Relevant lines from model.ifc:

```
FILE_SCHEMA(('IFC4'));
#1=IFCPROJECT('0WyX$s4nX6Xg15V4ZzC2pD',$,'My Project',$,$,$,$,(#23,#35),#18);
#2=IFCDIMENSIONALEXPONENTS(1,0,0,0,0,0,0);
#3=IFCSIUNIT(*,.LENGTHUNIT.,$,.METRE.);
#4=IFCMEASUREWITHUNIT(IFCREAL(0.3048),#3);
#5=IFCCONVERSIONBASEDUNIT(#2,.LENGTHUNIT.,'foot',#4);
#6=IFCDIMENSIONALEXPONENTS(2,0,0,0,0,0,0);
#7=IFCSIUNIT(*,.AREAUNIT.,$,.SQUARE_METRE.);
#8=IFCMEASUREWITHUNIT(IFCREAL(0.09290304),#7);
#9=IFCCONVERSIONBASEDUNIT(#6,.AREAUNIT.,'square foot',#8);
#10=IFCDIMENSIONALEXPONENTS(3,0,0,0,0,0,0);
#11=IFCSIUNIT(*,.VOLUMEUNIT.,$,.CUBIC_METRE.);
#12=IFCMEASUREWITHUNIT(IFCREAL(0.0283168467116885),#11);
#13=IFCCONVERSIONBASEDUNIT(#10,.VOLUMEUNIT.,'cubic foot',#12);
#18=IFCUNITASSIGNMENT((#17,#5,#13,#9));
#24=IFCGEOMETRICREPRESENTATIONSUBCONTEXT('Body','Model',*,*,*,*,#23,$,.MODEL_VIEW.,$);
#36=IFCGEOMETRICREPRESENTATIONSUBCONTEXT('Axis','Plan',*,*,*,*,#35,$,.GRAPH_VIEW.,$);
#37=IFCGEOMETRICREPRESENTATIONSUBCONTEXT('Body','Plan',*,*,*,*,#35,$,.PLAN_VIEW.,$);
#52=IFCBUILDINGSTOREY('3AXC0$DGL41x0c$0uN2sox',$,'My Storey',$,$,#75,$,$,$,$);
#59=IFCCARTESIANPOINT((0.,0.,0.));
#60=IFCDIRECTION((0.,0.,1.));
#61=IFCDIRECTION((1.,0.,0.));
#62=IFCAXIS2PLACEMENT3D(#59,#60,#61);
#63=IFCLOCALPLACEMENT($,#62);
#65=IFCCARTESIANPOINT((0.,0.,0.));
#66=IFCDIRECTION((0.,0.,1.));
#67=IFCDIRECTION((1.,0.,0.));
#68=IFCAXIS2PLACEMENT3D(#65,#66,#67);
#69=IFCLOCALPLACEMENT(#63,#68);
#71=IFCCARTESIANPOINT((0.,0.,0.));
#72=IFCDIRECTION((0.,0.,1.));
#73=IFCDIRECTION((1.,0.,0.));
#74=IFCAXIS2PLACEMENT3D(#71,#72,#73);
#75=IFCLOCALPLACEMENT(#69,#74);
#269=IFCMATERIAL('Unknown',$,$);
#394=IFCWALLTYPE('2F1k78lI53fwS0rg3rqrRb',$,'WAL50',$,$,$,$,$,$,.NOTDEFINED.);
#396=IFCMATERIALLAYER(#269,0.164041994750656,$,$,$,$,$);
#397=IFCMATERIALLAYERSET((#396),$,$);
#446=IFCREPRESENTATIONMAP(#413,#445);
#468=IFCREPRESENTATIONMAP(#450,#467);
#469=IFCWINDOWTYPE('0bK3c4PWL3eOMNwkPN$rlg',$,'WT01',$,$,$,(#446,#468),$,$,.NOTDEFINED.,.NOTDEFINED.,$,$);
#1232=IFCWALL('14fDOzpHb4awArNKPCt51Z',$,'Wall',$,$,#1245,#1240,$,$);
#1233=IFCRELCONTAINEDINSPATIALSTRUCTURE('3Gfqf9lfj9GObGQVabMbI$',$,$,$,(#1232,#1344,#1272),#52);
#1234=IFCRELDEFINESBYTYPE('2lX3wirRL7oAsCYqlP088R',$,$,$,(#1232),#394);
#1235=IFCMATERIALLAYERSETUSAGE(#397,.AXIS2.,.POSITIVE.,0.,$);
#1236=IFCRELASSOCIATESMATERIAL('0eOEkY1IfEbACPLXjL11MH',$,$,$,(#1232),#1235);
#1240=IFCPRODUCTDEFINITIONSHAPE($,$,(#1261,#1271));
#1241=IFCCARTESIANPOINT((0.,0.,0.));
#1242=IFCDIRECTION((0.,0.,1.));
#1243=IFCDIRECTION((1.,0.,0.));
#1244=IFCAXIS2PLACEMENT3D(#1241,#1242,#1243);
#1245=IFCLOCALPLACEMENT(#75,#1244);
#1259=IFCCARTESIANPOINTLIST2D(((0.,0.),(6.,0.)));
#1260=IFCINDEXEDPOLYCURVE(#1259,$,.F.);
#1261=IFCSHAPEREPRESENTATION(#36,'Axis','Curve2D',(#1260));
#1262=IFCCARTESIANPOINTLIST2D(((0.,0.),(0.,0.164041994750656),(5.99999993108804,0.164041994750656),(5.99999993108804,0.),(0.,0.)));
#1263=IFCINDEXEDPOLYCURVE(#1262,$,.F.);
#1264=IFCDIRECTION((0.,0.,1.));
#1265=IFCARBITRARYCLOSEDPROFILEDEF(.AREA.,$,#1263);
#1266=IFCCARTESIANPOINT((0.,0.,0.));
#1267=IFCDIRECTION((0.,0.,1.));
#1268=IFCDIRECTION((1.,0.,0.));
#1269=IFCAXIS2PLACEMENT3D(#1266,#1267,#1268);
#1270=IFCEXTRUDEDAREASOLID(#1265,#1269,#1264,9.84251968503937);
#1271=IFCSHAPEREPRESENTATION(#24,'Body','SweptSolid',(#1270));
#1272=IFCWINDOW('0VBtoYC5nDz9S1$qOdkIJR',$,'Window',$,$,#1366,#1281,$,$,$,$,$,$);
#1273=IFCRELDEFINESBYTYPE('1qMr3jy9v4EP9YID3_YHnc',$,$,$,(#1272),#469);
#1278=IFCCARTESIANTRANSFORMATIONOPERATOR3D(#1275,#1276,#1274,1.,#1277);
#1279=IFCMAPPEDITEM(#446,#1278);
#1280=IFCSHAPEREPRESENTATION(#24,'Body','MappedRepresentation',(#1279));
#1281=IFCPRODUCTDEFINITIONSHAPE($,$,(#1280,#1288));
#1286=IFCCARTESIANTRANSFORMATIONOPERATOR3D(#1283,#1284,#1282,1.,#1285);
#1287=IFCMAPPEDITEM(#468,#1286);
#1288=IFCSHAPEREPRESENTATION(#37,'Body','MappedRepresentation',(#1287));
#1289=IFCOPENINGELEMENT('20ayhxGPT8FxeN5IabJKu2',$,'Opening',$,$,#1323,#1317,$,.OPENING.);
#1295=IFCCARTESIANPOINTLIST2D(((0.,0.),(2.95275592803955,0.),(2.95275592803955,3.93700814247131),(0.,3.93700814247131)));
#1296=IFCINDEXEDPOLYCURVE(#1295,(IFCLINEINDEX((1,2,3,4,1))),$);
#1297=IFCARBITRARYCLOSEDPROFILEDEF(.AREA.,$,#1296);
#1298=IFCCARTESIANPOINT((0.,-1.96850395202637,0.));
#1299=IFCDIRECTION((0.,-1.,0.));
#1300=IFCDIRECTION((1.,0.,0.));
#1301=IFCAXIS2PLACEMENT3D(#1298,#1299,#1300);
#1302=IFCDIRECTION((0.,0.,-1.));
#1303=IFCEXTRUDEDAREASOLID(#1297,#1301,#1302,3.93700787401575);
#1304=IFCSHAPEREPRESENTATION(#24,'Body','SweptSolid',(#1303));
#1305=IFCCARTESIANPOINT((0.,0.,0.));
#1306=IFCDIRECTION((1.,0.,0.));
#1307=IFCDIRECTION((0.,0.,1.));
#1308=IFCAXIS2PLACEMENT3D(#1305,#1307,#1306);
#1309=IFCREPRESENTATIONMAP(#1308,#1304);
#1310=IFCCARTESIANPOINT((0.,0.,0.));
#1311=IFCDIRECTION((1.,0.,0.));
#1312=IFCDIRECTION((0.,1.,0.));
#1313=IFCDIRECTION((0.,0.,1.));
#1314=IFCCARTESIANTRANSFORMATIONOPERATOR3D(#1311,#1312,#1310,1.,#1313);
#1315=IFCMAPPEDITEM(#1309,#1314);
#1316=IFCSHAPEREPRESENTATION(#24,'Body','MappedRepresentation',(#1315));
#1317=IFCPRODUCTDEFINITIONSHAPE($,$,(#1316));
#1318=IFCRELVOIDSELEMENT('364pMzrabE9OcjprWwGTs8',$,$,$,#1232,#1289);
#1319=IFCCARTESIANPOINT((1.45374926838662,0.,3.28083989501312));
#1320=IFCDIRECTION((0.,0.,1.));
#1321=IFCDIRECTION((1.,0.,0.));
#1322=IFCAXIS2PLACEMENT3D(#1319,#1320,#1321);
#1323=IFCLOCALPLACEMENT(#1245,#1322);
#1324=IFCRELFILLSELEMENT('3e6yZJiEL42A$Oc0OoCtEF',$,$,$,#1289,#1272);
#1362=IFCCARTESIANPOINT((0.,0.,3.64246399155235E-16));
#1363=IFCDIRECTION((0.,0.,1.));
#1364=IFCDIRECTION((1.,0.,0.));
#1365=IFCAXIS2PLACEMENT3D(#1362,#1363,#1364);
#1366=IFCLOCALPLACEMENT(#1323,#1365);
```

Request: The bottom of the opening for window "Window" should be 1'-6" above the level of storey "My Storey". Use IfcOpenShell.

```python
import numpy as np
import ifcopenshell
import ifcopenshell.api.geometry
import ifcopenshell.geom
import ifcopenshell.util.element
import ifcopenshell.util.placement
import ifcopenshell.util.shape
import ifcopenshell.util.unit

model = ifcopenshell.open("model.ifc")
unit_scale = ifcopenshell.util.unit.calculate_unit_scale(model)

window = model.by_guid("0VBtoYC5nDz9S1$qOdkIJR")
opening = window.FillsVoids[0].RelatingOpeningElement
storey = ifcopenshell.util.element.get_container(window, ifc_class="IfcBuildingStorey")
level = ifcopenshell.util.placement.get_local_placement(storey.ObjectPlacement)[2, 3]

# The opening's origin need not be at the sill, so measure its lowest point.
shape = ifcopenshell.geom.create_shape(ifcopenshell.geom.settings(), opening)
bottom = ifcopenshell.util.shape.get_shape_bottom_elevation(shape, shape.geometry) / unit_scale
dz = level + 18 * 0.0254 / unit_scale - bottom

shift = np.array([0.0, 0.0, dz])
# The window is placed relative to its opening, so it follows when the opening moves.
matrix = ifcopenshell.util.placement.get_local_placement(opening.ObjectPlacement)
matrix[:3, 3] += shift
ifcopenshell.api.geometry.edit_object_placement(
    model, product=opening, matrix=matrix, is_si=False, should_transform_children=True
)

print(f"moved by {dz * unit_scale:+.3f} m")

model.write("model_updated.ifc")
```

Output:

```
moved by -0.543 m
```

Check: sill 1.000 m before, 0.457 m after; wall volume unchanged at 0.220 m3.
